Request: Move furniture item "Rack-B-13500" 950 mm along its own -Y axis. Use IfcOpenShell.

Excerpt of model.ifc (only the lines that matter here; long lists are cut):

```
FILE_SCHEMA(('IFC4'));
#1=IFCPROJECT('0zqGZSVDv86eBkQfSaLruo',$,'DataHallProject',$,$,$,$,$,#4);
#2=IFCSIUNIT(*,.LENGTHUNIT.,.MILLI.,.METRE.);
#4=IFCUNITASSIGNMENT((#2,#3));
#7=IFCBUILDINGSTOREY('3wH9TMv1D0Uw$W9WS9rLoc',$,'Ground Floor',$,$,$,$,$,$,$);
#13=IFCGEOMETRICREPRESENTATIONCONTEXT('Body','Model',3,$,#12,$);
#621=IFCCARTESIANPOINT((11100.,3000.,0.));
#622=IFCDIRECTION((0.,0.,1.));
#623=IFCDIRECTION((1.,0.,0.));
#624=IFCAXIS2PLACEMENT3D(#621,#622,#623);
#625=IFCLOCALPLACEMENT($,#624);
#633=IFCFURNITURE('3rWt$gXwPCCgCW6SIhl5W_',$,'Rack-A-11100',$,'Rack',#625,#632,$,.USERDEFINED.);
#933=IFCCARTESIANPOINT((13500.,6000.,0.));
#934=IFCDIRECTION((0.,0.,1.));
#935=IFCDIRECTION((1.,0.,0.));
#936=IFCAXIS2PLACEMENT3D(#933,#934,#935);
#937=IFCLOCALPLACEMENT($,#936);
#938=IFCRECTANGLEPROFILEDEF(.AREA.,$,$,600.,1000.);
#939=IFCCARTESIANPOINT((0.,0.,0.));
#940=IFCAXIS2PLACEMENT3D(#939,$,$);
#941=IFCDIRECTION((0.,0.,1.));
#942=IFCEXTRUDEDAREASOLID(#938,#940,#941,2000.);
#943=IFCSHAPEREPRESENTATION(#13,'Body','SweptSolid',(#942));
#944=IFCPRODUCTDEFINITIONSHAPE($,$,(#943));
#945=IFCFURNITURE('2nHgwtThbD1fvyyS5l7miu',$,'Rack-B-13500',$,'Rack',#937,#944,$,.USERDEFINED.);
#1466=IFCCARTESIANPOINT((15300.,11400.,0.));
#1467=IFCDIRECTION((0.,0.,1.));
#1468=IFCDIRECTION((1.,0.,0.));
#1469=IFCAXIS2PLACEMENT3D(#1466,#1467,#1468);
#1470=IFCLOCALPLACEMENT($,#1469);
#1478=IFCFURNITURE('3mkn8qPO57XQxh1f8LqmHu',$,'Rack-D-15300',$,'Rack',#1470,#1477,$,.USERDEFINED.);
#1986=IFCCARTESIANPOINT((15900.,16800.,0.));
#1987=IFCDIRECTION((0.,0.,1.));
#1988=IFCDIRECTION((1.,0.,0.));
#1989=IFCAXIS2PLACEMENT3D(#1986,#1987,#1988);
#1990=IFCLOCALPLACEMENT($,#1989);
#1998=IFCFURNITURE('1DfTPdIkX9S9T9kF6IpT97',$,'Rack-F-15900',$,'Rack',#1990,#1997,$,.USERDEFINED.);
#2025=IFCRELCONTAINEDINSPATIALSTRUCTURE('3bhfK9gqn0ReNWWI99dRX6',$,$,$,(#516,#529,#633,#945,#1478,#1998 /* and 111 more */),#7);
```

```python
import ifcopenshell
import ifcopenshell.api.geometry
import ifcopenshell.util.placement
import ifcopenshell.util.unit

model = ifcopenshell.open("model.ifc")
unit_scale = ifcopenshell.util.unit.calculate_unit_scale(model)

item = model.by_guid("2nHgwtThbD1fvyyS5l7miu")
matrix = ifcopenshell.util.placement.get_local_placement(item.ObjectPlacement)
matrix[:3, 3] -= matrix[:3, 1] * 0.95 / unit_scale
ifcopenshell.api.geometry.edit_object_placement(model, product=item, matrix=matrix, is_si=False)

print(ifcopenshell.util.placement.get_local_placement(item.ObjectPlacement).round(3) + 0.0)

model.write("model_edited.ifc")
```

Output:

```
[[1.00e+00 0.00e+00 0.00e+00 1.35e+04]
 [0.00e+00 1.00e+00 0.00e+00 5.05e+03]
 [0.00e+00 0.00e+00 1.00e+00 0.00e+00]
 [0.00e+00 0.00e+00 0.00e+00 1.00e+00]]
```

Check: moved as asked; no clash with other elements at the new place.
